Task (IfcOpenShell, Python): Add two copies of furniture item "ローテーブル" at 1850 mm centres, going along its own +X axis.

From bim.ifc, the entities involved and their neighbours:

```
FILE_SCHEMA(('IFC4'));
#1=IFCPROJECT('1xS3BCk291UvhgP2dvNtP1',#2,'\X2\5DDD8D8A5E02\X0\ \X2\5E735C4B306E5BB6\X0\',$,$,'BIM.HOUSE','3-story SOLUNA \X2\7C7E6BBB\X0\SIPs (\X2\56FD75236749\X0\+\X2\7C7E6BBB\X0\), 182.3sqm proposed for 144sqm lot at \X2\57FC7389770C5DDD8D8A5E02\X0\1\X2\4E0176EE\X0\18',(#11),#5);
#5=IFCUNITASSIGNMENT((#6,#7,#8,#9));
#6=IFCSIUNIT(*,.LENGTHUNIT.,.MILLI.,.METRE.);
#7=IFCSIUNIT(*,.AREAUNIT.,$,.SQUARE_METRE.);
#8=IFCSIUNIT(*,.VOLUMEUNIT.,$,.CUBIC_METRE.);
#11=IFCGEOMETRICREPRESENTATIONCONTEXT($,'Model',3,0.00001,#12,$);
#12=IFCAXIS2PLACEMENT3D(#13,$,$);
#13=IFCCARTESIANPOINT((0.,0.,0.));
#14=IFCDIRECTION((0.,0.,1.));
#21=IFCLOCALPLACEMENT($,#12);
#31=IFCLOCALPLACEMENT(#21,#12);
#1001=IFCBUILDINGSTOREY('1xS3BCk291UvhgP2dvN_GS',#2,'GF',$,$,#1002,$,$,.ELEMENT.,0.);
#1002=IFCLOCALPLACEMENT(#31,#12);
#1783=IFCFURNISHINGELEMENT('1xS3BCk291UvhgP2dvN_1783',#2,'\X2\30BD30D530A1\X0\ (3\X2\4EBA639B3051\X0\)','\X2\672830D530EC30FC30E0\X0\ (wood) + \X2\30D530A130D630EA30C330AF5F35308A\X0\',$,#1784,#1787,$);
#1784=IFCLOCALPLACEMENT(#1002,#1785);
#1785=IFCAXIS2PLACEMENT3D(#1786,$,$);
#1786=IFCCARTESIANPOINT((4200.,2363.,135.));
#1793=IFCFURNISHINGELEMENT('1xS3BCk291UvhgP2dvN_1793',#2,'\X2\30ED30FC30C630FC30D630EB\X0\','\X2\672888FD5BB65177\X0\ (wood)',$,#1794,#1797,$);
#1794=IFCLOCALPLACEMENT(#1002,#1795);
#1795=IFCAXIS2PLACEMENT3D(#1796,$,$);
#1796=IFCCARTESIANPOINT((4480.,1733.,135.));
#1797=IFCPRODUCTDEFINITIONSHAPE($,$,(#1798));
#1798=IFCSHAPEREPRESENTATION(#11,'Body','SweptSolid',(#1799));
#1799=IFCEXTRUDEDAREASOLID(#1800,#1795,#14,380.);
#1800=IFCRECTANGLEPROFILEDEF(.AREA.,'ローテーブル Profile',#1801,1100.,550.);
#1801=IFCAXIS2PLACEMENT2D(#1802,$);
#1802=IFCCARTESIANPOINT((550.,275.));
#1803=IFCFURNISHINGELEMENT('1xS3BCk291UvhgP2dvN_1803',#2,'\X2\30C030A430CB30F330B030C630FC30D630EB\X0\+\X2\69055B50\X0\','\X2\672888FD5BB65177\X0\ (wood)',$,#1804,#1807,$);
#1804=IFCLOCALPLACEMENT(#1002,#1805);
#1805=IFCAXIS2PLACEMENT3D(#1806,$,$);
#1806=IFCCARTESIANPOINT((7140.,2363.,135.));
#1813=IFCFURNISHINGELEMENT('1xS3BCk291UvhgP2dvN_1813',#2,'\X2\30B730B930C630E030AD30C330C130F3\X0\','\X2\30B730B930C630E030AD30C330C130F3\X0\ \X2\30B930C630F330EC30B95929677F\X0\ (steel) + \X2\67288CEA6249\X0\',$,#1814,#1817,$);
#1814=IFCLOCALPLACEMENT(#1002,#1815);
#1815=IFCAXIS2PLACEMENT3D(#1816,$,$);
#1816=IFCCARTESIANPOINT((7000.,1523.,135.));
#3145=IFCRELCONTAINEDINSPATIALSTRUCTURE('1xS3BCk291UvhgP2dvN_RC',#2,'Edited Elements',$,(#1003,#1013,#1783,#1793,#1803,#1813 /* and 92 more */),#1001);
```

```python
import ifcopenshell
import ifcopenshell.api.geometry
import ifcopenshell.api.root
import ifcopenshell.util.element
import ifcopenshell.util.placement
import ifcopenshell.util.unit

model = ifcopenshell.open("bim.ifc")
unit_scale = ifcopenshell.util.unit.calculate_unit_scale(model)


def reuse_history(source, copy):
    """copy_class also copies each property set's owner history, people and application; keep the originals."""
    for rel in copy.IsDefinedBy:
        if rel.is_a("IfcRelDefinesByProperties") and (history := rel.RelatingPropertyDefinition.OwnerHistory):
            rel.RelatingPropertyDefinition.OwnerHistory = source.OwnerHistory
            ifcopenshell.util.element.remove_deep2(model, history)


source = model.by_guid("1xS3BCk291UvhgP2dvN_1793")
base = ifcopenshell.util.placement.get_local_placement(source.ObjectPlacement)
step = base[:3, 0] * 1.85 / unit_scale

for i in range(1, 3):
    copy = ifcopenshell.api.root.copy_class(model, product=source)
    copy.Representation = ifcopenshell.util.element.copy_deep(
        model, source.Representation, exclude=["IfcGeometricRepresentationContext", "IfcRepresentationMap"]
    )
    reuse_history(source, copy)
    matrix = base.copy()
    matrix[:3, 3] += i * step
    print("added at", matrix[:3, 3].round(3) + 0.0)
    ifcopenshell.api.geometry.edit_object_placement(model, product=copy, matrix=matrix, is_si=False)

model.write("bim_updated.ifc")
```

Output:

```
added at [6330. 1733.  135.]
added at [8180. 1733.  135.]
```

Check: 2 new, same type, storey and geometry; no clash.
